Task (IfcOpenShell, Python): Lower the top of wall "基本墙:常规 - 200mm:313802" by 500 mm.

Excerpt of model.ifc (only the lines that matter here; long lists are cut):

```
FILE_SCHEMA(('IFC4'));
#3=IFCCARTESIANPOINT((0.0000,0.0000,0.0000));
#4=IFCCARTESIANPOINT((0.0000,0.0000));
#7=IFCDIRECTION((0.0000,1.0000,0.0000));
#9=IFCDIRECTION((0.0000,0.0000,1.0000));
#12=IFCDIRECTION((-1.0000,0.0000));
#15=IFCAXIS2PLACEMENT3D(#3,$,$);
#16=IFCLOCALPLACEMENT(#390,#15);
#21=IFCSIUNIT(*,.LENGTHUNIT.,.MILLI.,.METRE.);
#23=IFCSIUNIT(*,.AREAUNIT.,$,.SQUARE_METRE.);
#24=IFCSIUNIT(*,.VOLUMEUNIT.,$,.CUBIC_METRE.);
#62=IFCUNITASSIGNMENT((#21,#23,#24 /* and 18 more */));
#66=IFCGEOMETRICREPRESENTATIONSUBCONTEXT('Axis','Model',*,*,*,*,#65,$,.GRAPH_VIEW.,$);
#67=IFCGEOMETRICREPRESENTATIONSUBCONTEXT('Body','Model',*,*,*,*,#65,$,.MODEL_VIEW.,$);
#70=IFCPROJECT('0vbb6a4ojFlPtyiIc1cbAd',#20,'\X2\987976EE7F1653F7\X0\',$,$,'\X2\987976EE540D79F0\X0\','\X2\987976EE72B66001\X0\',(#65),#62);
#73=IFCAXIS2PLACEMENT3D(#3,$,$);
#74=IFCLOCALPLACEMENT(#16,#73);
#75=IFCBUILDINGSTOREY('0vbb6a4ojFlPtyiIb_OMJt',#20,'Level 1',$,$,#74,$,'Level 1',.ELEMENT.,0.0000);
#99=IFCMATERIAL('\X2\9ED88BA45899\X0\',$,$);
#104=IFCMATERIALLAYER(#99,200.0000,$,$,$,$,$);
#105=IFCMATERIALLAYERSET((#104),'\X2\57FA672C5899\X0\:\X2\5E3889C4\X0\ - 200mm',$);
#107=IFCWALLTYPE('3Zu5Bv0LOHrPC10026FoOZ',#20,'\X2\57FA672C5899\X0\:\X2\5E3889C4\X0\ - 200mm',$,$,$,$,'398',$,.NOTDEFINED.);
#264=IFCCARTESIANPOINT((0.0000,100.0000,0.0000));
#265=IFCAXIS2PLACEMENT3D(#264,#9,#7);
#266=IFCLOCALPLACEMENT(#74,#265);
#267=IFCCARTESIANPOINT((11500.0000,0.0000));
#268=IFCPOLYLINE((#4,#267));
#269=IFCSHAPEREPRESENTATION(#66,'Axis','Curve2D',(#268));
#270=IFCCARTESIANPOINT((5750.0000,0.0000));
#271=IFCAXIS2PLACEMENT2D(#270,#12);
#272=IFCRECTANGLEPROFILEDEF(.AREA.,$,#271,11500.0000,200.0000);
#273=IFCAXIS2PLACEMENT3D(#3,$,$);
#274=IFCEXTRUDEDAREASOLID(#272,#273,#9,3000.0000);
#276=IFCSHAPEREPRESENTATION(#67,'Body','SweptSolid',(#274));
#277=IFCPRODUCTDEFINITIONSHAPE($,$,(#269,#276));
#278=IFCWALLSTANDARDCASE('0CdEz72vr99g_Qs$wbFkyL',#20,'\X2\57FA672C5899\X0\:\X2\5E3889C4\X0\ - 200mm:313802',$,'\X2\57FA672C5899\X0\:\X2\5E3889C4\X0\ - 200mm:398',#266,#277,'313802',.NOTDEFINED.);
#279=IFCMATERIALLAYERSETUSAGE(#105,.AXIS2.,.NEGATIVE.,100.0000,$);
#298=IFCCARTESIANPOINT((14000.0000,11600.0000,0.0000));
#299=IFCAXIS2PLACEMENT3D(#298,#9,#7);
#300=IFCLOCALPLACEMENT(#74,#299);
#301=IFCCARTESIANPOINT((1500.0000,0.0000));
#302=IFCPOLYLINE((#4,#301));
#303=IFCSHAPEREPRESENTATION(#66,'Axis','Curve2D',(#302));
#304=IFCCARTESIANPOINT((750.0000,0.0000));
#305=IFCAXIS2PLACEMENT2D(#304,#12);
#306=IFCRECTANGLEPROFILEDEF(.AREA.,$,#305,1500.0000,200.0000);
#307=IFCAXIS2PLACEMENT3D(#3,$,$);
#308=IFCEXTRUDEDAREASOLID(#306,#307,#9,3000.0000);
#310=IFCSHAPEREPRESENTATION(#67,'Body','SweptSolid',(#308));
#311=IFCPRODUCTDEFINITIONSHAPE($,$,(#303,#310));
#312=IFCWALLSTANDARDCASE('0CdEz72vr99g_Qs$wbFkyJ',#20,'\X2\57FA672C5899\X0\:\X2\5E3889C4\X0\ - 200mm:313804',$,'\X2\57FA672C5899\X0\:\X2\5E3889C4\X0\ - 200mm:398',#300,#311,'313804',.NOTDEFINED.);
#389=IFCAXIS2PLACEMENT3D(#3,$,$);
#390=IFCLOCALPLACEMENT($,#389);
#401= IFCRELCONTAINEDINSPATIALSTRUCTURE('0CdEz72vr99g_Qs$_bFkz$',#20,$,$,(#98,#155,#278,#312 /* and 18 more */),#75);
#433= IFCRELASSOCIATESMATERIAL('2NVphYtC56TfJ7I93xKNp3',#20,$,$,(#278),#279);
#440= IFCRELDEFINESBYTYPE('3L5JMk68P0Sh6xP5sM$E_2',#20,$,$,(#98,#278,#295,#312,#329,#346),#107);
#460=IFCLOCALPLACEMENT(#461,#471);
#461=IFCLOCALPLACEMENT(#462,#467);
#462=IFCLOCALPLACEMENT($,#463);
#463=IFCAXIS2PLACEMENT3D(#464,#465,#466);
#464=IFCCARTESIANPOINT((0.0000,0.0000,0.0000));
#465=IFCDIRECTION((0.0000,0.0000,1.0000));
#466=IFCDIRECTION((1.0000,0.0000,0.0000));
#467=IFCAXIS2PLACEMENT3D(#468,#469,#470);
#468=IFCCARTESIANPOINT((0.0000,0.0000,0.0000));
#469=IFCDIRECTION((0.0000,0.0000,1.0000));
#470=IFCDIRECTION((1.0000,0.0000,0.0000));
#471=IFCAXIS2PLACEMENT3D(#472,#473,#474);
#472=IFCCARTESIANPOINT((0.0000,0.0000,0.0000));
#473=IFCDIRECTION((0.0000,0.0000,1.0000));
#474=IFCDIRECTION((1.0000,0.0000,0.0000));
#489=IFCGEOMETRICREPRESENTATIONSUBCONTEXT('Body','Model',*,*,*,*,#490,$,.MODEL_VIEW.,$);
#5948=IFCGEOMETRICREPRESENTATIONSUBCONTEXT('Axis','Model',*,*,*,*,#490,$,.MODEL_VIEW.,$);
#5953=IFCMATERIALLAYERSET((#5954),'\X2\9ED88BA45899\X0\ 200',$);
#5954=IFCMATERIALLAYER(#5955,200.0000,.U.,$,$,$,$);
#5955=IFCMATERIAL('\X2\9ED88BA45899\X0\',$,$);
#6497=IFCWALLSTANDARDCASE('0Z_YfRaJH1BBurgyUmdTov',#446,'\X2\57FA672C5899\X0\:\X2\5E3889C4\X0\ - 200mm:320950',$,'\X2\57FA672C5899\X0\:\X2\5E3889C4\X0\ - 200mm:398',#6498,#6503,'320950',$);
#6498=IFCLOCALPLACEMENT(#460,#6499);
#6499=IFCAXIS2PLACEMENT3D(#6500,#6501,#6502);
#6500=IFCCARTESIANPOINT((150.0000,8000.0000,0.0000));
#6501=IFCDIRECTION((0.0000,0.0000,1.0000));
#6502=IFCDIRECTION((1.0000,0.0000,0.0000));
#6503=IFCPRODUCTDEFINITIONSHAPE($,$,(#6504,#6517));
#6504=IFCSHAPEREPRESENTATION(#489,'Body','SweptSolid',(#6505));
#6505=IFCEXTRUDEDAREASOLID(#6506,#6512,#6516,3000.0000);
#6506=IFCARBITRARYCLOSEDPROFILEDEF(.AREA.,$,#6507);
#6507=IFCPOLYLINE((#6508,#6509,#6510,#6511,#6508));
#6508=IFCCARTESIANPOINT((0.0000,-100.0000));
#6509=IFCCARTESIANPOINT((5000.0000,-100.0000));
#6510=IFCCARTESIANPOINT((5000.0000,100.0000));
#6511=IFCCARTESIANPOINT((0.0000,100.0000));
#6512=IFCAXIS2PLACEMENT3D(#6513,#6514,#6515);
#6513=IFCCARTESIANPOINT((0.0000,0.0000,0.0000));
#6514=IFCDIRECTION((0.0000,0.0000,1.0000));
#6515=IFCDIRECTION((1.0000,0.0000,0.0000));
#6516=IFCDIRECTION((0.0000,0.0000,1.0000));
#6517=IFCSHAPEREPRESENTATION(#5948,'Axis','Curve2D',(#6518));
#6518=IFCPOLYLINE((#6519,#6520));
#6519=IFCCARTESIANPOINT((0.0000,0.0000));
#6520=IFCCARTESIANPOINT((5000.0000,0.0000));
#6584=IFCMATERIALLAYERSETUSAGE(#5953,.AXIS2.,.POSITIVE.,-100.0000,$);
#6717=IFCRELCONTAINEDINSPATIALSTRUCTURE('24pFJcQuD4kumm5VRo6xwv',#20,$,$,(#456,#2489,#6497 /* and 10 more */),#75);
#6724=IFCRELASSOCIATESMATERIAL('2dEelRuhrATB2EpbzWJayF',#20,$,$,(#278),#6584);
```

```python
import ifcopenshell
import ifcopenshell.geom
import ifcopenshell.util.representation
import ifcopenshell.util.shape

model = ifcopenshell.open("model.ifc")
settings = ifcopenshell.geom.settings()


def volume(element):
    """Net volume in cubic metres, openings subtracted."""
    shape = ifcopenshell.geom.create_shape(settings, element)
    return ifcopenshell.util.shape.get_volume(shape.geometry)


wall = model.by_guid("0CdEz72vr99g_Qs$wbFkyL")
before = volume(wall)

body = ifcopenshell.util.representation.get_representation(wall, "Model", "Body")
solid = body.Items[0]
old_height = solid.Depth
solid.Depth -= 500.0
after = volume(wall)

print(f"height {old_height:g} -> {solid.Depth:g}, volume {before:.3f} -> {after:.3f} m3")

model.write("model_edited.ifc")
```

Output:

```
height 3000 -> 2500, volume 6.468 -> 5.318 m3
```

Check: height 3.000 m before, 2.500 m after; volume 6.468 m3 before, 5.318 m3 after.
